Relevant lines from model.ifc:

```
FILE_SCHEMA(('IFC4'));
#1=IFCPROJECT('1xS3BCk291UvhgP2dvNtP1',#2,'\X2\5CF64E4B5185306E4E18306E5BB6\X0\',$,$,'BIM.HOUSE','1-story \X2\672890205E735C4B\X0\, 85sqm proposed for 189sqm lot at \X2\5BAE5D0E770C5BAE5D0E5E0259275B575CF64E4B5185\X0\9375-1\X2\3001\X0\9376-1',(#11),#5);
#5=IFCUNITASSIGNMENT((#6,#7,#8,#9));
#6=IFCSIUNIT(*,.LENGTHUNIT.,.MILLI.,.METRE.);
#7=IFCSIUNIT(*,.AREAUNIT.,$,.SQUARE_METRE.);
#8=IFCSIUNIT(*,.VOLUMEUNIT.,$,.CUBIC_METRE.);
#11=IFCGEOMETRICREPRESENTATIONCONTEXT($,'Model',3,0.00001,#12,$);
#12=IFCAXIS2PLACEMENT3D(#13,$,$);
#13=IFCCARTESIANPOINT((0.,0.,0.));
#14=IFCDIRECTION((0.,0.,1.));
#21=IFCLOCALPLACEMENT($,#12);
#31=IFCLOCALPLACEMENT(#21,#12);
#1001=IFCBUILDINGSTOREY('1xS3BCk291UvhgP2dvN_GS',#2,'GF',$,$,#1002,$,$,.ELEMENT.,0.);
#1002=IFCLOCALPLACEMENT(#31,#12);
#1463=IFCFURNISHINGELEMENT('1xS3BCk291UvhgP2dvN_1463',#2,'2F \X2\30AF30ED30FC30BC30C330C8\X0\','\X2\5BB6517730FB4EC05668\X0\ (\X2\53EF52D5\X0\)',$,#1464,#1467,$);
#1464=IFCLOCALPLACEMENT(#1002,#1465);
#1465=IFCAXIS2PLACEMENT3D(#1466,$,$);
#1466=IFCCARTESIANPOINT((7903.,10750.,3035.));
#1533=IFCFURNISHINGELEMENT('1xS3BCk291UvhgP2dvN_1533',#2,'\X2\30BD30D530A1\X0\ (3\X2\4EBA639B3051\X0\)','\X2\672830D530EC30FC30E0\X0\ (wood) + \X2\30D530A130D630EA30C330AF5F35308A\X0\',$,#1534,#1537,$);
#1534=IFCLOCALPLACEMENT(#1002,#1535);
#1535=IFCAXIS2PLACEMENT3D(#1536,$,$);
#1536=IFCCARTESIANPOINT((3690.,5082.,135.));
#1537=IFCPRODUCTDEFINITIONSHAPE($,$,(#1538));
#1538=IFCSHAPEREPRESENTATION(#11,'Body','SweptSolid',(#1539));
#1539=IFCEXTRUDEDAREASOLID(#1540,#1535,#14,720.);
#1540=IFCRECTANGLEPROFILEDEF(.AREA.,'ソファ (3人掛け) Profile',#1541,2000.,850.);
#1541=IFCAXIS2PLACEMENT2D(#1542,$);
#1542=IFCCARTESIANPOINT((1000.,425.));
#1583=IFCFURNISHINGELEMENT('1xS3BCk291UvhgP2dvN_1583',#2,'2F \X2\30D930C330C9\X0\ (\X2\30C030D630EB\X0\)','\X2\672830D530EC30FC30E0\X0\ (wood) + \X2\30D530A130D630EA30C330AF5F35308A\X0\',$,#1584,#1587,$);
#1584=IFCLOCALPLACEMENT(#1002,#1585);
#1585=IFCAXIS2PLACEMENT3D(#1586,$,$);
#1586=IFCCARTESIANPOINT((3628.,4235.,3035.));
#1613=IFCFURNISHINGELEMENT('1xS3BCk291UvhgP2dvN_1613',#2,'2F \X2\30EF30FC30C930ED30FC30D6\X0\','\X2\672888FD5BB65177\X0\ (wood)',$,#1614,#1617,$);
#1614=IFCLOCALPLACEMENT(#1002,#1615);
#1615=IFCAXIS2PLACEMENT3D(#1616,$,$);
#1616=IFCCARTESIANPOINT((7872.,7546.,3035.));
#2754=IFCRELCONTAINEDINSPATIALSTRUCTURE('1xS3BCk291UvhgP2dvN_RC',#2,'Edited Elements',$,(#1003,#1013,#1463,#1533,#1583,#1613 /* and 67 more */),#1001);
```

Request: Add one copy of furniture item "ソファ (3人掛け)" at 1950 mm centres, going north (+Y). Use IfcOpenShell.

```python
import numpy as np
import ifcopenshell
import ifcopenshell.api.geometry
import ifcopenshell.api.root
import ifcopenshell.util.element
import ifcopenshell.util.placement
import ifcopenshell.util.unit

model = ifcopenshell.open("model.ifc")
unit_scale = ifcopenshell.util.unit.calculate_unit_scale(model)


def reuse_history(source, copy):
    """copy_class also copies each property set's owner history, people and application; keep the originals."""
    for rel in copy.IsDefinedBy:
        if rel.is_a("IfcRelDefinesByProperties") and (history := rel.RelatingPropertyDefinition.OwnerHistory):
            rel.RelatingPropertyDefinition.OwnerHistory = source.OwnerHistory
            ifcopenshell.util.element.remove_deep2(model, history)


source = model.by_guid("1xS3BCk291UvhgP2dvN_1533")
base = ifcopenshell.util.placement.get_local_placement(source.ObjectPlacement)
step = np.array([0.0, 1.0, 0.0]) * 1.95 / unit_scale

for i in range(1, 2):
    copy = ifcopenshell.api.root.copy_class(model, product=source)
    copy.Representation = ifcopenshell.util.element.copy_deep(
        model, source.Representation, exclude=["IfcGeometricRepresentationContext", "IfcRepresentationMap"]
    )
    reuse_history(source, copy)
    matrix = base.copy()
    matrix[:3, 3] += i * step
    print("added at", matrix[:3, 3].round(3) + 0.0)
    ifcopenshell.api.geometry.edit_object_placement(model, product=copy, matrix=matrix, is_si=False)

model.write("model-out.ifc")
```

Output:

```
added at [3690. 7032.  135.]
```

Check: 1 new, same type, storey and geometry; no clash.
